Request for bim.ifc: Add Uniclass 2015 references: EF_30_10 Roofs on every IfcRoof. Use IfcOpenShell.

First a look at what the model holds.

```python
import ifcopenshell

model = ifcopenshell.open("bim.ifc")
print(model.schema)
print("classifications:", [c.Name for c in model.by_type("IfcClassification")])
for ifc_class in ("IfcDoor", "IfcRoof", "IfcStair", "IfcWall", "IfcWindow"):
    print(ifc_class, len(model.by_type(ifc_class)))
```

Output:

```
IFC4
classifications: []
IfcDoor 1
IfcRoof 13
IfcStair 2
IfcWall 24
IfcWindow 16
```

```python
import ifcopenshell
import ifcopenshell.api.classification

model = ifcopenshell.open("bim.ifc")

system = ifcopenshell.api.classification.add_classification(model, classification="Uniclass 2015")

codes = {
    "IfcRoof": ("EF_30_10", "Roofs"),
}
for ifc_class, (code, name) in codes.items():
    products = model.by_type(ifc_class)
    ifcopenshell.api.classification.add_reference(
        model, products=products, classification=system, identification=code, name=name
    )
    print(code, len(products))

model.write("bim_rev.ifc")
```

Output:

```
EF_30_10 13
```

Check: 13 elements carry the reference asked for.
